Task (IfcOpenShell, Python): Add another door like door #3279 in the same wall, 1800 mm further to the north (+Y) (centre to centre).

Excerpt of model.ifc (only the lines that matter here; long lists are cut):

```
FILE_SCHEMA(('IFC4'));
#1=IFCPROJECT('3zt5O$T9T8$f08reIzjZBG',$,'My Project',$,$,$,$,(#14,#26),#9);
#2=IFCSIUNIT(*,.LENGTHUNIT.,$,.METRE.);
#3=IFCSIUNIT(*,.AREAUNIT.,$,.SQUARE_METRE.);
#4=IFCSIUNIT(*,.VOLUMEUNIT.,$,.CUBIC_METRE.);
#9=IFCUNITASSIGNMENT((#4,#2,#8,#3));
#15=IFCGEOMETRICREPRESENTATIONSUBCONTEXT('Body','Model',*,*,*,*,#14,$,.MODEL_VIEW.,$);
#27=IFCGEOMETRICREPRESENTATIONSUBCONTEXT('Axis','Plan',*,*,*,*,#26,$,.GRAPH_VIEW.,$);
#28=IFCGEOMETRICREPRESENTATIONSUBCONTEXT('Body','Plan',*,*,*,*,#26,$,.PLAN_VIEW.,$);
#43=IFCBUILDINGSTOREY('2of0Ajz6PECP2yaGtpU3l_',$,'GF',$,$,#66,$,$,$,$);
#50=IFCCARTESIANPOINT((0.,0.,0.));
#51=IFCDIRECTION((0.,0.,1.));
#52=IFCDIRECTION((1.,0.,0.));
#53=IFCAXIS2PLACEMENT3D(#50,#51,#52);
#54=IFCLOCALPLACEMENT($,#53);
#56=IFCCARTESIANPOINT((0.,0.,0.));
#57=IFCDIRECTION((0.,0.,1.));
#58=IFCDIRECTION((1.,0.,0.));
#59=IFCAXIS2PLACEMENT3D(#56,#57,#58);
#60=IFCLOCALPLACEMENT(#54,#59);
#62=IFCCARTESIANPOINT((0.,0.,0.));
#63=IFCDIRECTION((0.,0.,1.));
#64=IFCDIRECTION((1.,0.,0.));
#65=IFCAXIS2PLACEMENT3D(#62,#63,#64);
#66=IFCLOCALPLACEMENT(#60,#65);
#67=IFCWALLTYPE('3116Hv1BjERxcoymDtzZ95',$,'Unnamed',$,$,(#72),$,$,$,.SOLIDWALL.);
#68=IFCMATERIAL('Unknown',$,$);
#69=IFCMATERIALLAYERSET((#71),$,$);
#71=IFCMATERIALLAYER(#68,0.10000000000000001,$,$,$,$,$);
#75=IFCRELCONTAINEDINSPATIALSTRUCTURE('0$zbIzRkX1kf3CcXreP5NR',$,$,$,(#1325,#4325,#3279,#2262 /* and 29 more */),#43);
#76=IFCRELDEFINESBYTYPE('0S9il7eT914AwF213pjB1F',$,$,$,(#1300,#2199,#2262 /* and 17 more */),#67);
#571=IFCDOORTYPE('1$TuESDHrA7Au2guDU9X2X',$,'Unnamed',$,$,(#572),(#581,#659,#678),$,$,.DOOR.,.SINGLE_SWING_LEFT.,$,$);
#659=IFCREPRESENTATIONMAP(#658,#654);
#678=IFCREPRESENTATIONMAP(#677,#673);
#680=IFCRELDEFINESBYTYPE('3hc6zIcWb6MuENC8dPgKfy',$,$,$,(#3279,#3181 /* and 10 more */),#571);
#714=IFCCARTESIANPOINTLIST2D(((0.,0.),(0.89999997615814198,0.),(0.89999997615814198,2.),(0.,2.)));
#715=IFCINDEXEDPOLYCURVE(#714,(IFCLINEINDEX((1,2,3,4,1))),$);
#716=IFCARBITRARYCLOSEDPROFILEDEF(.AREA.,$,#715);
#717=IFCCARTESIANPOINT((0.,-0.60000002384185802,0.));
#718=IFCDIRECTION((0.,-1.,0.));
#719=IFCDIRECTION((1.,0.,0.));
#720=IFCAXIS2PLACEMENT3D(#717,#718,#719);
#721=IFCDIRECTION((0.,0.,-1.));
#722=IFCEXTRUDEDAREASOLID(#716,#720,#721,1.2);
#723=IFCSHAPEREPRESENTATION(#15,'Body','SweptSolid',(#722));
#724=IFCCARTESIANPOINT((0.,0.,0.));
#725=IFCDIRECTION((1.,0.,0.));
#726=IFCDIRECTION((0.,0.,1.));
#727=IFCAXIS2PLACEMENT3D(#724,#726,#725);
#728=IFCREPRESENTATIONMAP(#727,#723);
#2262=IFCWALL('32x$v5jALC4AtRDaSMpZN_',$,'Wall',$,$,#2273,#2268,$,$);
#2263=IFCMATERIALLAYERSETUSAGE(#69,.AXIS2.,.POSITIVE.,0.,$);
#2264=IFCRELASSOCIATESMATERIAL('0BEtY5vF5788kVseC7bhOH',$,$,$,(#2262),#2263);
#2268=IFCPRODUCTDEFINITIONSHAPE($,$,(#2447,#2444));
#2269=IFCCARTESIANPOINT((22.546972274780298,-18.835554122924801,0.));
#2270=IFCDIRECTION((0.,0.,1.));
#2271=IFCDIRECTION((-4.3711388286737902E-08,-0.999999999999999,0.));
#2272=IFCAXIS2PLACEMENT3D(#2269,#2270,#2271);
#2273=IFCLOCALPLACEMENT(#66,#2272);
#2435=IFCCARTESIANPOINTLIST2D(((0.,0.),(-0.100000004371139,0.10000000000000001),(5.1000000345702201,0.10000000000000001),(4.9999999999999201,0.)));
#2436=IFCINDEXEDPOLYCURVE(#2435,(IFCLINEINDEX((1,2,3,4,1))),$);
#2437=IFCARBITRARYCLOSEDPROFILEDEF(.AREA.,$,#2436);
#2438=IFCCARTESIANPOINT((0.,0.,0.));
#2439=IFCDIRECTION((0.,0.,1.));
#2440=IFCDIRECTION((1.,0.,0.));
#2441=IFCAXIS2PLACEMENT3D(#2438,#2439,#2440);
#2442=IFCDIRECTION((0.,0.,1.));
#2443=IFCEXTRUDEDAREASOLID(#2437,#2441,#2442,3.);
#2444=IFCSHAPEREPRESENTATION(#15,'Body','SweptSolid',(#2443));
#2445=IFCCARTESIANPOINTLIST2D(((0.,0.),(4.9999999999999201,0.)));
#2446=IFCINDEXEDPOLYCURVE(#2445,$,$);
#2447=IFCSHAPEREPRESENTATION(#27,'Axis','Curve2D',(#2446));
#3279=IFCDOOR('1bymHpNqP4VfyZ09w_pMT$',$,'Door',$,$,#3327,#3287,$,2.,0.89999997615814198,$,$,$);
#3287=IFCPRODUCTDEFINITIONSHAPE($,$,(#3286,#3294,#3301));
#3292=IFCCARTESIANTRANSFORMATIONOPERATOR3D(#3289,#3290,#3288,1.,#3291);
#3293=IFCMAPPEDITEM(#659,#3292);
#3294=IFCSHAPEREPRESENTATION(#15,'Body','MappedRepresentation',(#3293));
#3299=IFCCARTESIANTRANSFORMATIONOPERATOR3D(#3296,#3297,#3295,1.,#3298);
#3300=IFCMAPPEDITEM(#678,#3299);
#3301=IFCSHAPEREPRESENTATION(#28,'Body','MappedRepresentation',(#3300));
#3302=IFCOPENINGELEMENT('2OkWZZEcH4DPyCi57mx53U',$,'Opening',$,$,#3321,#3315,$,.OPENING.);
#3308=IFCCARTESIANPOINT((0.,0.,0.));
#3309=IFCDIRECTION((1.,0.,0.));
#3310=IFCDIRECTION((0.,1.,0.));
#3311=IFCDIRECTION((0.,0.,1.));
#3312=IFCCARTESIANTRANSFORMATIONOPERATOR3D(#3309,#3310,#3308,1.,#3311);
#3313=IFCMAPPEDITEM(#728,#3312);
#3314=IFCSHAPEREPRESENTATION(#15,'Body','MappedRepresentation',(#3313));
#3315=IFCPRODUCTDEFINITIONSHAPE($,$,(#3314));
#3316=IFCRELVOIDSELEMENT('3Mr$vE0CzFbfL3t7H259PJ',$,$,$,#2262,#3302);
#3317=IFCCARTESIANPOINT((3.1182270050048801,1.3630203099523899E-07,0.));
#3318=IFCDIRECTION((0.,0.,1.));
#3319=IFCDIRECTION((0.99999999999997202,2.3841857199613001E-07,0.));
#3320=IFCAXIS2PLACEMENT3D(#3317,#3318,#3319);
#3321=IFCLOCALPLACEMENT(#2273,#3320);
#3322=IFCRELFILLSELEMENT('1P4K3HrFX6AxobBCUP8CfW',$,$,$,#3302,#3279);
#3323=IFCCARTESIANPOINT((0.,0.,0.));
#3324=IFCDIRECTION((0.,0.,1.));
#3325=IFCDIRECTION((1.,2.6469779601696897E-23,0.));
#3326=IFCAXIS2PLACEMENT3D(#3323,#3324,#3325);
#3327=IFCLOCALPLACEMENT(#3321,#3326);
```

```python
import ifcopenshell
import ifcopenshell.api.feature
import ifcopenshell.api.geometry
import ifcopenshell.api.root
import ifcopenshell.geom
import ifcopenshell.util.element
import ifcopenshell.util.placement
import ifcopenshell.util.shape
import ifcopenshell.util.unit

model = ifcopenshell.open("model.ifc")
unit_scale = ifcopenshell.util.unit.calculate_unit_scale(model)
settings = ifcopenshell.geom.settings()


def volume(element):
    """Net volume in cubic metres, openings subtracted."""
    shape = ifcopenshell.geom.create_shape(settings, element)
    return ifcopenshell.util.shape.get_volume(shape.geometry)


door = model.by_guid("1bymHpNqP4VfyZ09w_pMT$")
opening = door.FillsVoids[0].RelatingOpeningElement
wall = opening.VoidsElements[0].RelatingBuildingElement
before = volume(wall)
shift = ifcopenshell.util.placement.get_local_placement(wall.ObjectPlacement)[:3, 0] * -1.8 / unit_scale

# copy_class copies the void relationship, type, container and properties, but no geometry.
new_opening = ifcopenshell.api.root.copy_class(model, product=opening)
new_opening.Representation = ifcopenshell.util.element.copy_deep(
    model, opening.Representation, exclude=["IfcGeometricRepresentationContext", "IfcRepresentationMap"]
)
new_door = ifcopenshell.api.root.copy_class(model, product=door)
new_door.Representation = ifcopenshell.util.element.copy_deep(
    model, door.Representation, exclude=["IfcGeometricRepresentationContext", "IfcRepresentationMap"]
)
ifcopenshell.api.feature.add_filling(model, opening=new_opening, element=new_door)

for old, new in ((opening, new_opening), (door, new_door)):
    matrix = ifcopenshell.util.placement.get_local_placement(old.ObjectPlacement)
    matrix[:3, 3] += shift
    ifcopenshell.api.geometry.edit_object_placement(model, product=new, matrix=matrix, is_si=False)

after = volume(wall)

print(f"wall volume {before:.3f} -> {after:.3f} m3")

model.write("model_updated.ifc")
```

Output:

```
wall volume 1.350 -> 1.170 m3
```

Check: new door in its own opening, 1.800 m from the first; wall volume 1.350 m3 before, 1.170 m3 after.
